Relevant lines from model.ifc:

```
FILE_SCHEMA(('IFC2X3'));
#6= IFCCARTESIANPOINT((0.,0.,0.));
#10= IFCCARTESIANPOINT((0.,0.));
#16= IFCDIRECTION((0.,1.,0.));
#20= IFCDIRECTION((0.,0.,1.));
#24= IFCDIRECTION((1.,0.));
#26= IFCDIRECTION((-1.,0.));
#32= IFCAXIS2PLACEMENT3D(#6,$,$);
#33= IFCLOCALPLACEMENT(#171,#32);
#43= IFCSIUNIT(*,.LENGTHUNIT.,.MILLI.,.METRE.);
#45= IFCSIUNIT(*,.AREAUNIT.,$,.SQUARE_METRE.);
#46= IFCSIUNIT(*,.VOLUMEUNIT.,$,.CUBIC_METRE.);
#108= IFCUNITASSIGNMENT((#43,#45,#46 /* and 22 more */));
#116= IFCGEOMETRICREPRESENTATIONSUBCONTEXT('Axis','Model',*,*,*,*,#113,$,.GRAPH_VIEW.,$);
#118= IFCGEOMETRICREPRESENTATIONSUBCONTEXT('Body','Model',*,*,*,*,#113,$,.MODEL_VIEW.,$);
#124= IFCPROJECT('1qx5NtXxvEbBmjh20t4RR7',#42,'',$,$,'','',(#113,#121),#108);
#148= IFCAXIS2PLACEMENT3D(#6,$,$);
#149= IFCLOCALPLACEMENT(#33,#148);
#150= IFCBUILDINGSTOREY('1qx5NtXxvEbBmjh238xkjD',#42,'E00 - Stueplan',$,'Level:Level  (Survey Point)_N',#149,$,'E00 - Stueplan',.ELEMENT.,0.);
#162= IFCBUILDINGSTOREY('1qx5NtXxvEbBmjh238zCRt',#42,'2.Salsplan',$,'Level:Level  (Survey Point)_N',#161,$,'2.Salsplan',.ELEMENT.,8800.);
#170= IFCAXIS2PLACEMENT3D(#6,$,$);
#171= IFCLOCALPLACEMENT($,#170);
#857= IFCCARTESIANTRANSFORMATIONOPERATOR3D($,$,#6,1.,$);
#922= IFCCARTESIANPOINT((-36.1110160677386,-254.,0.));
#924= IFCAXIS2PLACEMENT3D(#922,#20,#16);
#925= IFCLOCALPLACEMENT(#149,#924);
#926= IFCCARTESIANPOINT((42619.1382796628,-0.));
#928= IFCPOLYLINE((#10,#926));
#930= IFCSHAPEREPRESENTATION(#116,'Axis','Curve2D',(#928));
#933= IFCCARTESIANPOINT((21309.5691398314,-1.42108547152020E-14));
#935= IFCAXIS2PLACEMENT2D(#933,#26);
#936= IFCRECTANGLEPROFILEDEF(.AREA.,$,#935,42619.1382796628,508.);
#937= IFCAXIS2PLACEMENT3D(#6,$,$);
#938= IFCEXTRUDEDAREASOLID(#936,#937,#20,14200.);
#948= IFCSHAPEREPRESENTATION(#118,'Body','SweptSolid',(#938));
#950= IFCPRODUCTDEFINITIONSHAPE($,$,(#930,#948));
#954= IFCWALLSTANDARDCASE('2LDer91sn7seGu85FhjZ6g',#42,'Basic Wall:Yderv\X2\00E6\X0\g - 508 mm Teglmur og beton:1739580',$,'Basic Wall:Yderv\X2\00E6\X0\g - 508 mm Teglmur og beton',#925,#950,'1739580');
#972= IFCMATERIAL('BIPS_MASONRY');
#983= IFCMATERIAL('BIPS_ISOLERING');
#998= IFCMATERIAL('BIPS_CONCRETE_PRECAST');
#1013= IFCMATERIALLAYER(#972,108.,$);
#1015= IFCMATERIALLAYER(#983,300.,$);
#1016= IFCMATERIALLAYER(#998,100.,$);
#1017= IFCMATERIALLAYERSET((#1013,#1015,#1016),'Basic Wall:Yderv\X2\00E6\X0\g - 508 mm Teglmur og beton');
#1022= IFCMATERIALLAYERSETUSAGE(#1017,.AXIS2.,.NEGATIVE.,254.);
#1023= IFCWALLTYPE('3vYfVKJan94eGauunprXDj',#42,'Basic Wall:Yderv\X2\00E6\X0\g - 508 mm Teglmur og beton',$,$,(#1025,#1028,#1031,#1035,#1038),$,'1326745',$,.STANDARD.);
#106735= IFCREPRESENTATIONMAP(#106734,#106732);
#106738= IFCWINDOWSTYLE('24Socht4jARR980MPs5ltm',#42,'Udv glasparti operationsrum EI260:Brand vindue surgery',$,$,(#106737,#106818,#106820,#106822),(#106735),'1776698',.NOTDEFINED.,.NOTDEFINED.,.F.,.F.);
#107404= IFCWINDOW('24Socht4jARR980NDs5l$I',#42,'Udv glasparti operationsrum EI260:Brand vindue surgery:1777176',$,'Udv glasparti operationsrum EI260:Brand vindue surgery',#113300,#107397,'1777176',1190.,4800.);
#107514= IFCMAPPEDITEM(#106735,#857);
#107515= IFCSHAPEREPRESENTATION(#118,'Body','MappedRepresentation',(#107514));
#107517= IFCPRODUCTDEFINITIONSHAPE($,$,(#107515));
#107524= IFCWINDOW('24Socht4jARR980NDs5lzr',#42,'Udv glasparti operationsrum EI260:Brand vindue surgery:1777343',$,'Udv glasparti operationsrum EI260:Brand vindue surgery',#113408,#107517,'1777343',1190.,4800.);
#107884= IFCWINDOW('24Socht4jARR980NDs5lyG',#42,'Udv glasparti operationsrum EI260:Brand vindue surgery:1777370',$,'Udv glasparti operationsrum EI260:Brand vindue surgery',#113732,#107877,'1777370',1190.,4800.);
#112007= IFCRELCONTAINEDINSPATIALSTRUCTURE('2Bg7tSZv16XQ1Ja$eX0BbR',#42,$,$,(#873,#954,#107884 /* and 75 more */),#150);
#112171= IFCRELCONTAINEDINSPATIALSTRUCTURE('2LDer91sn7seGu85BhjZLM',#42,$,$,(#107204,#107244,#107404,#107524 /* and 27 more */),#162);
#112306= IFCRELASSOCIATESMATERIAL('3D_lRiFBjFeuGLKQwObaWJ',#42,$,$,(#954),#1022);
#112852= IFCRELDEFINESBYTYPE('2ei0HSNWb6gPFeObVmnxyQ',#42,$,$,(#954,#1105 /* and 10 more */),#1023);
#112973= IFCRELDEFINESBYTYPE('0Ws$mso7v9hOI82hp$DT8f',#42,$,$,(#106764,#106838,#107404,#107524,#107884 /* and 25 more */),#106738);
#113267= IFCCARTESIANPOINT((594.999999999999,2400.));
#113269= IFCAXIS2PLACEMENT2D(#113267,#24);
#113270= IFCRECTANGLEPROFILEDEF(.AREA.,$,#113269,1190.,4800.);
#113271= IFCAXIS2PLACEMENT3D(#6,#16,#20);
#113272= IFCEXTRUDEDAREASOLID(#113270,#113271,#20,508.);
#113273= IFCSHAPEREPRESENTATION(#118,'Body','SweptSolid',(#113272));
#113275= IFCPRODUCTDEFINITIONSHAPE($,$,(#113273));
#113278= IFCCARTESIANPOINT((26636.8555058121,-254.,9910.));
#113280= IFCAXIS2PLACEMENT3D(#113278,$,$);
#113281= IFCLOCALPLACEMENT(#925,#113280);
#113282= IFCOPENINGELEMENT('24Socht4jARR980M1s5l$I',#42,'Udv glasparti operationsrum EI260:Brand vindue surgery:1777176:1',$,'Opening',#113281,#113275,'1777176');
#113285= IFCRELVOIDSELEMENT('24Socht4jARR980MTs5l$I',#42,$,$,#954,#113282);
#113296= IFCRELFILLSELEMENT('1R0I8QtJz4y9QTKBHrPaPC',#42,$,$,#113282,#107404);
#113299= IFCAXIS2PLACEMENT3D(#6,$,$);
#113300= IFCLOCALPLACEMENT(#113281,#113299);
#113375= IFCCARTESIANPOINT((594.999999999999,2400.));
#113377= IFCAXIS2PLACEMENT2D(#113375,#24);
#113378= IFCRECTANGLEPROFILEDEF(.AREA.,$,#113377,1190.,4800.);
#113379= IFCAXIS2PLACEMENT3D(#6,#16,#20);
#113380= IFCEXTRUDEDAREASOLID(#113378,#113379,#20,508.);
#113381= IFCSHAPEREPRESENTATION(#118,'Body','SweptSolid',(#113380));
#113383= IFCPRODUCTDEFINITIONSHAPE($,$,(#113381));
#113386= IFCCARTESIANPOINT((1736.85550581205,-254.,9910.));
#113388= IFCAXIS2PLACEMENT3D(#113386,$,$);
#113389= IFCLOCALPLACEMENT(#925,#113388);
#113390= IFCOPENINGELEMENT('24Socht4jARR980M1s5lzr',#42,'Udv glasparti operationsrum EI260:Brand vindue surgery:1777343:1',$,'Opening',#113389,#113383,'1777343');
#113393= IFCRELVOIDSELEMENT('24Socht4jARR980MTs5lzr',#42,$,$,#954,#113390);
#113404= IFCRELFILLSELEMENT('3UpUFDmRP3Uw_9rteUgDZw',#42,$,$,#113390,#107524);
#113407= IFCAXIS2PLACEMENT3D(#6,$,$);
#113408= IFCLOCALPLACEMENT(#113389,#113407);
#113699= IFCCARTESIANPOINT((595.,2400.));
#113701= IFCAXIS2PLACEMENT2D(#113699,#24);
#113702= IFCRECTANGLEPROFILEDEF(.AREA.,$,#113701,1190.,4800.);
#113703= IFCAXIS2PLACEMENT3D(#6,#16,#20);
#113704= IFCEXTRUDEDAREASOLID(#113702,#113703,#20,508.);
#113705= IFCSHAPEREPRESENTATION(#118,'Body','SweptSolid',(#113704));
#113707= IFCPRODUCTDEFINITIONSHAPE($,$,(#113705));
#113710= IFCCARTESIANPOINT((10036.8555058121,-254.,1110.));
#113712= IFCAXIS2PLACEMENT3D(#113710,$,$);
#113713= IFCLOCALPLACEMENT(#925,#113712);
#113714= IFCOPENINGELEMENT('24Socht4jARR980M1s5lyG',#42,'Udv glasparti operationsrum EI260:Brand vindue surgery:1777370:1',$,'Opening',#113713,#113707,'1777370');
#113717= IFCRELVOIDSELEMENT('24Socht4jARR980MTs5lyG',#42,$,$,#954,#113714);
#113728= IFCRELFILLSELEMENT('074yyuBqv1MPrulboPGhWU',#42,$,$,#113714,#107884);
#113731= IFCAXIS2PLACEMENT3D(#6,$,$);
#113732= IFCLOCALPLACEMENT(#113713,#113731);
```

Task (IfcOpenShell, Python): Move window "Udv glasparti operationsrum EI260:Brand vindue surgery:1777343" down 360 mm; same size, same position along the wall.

```python
import numpy as np
import ifcopenshell
import ifcopenshell.api.geometry
import ifcopenshell.util.placement
import ifcopenshell.util.unit

model = ifcopenshell.open("model.ifc")
unit_scale = ifcopenshell.util.unit.calculate_unit_scale(model)

window = model.by_guid("24Socht4jARR980NDs5lzr")
opening = window.FillsVoids[0].RelatingOpeningElement
dz = -360.0

shift = np.array([0.0, 0.0, dz])
# The window is placed relative to its opening, so it follows when the opening moves.
matrix = ifcopenshell.util.placement.get_local_placement(opening.ObjectPlacement)
matrix[:3, 3] += shift
ifcopenshell.api.geometry.edit_object_placement(
    model, product=opening, matrix=matrix, is_si=False, should_transform_children=True
)

print(f"moved by {dz * unit_scale:+.3f} m")

model.write("model-out.ifc")
```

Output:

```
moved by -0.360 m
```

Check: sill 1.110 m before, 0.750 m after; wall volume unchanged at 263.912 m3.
